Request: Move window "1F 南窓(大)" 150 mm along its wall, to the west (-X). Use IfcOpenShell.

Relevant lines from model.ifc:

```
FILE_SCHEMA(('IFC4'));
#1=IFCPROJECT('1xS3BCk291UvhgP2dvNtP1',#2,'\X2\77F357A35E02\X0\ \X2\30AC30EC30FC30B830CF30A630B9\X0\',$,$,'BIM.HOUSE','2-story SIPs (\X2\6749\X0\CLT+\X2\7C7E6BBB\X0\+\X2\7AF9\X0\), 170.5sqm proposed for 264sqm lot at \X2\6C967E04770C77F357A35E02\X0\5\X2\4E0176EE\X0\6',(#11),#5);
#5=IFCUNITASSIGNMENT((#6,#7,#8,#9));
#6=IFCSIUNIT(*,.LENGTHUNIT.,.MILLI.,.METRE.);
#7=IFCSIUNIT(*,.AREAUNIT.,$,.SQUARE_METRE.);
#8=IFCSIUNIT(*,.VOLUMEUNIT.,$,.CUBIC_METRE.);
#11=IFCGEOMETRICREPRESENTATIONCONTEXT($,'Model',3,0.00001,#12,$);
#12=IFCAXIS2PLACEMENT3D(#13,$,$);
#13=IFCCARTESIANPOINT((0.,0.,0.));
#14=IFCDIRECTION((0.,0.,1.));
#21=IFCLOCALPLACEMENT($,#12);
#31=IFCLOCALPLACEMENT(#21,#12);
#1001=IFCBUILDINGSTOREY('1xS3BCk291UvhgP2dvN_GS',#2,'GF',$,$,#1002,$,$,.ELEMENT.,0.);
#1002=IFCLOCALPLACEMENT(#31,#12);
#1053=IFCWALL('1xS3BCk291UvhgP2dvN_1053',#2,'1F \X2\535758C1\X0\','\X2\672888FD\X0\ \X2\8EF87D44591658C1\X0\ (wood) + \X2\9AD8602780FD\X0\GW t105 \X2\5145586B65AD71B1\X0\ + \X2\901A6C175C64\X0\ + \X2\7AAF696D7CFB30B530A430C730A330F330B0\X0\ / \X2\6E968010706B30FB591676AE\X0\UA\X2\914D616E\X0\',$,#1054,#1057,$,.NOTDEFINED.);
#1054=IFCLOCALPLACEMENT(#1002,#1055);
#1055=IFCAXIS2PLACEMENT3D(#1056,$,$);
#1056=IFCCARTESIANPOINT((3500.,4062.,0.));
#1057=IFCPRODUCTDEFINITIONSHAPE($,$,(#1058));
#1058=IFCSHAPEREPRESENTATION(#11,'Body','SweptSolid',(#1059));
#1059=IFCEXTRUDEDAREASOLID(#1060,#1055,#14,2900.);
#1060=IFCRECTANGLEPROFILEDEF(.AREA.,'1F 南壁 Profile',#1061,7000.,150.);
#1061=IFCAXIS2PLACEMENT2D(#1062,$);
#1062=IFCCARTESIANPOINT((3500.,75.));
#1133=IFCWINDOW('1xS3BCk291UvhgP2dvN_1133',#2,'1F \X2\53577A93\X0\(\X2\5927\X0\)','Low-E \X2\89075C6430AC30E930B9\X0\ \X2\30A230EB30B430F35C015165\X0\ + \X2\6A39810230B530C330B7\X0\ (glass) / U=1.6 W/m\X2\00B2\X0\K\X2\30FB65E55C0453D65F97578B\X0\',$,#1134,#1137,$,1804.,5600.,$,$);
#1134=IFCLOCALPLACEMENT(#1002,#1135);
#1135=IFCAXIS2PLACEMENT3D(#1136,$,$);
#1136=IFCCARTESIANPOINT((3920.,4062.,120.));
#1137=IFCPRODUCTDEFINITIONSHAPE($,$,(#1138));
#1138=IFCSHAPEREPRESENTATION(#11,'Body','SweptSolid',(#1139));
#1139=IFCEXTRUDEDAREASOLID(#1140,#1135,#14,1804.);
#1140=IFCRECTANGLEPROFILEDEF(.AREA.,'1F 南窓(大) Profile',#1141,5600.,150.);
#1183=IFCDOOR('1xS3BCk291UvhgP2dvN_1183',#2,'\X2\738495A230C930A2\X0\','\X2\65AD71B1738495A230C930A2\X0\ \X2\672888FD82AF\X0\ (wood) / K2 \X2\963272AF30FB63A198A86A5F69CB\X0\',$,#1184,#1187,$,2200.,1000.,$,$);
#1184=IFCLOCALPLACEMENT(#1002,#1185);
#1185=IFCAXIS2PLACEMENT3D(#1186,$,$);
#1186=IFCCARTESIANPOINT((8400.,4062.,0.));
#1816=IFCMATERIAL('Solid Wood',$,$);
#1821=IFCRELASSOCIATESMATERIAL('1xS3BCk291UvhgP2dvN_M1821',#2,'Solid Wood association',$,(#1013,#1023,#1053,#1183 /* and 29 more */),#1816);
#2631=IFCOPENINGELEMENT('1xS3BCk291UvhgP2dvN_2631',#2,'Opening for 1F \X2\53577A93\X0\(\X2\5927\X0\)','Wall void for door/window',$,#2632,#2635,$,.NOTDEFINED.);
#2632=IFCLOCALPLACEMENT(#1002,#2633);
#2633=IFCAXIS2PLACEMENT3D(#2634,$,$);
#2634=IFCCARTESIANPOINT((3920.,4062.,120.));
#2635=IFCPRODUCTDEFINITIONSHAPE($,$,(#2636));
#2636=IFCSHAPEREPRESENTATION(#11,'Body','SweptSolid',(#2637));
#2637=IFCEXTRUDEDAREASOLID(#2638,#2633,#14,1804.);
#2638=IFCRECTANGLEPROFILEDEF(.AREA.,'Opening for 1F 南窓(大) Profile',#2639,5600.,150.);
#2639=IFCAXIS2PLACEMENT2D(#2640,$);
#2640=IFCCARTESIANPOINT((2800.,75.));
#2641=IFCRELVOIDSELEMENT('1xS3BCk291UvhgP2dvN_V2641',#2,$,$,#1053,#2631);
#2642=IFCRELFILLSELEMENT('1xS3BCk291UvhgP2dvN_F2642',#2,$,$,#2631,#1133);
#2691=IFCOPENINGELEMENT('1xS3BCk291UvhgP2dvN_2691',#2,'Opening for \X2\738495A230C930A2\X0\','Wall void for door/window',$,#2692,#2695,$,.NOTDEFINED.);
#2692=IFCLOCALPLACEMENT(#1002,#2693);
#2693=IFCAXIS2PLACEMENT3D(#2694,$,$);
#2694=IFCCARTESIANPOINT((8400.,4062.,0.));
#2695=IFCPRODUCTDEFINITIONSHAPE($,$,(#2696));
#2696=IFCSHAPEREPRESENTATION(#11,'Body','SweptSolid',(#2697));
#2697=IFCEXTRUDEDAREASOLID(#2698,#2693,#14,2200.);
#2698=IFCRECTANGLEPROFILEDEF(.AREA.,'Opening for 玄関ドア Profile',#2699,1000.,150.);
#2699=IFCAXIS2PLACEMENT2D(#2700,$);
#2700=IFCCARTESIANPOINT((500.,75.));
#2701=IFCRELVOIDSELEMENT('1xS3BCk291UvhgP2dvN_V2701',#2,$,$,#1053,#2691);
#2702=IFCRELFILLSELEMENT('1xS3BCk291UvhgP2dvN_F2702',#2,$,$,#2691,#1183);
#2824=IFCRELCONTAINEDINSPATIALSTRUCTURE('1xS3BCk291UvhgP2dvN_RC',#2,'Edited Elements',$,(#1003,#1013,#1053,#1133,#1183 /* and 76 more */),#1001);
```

```python
import ifcopenshell
import ifcopenshell.api.geometry
import ifcopenshell.util.placement

model = ifcopenshell.open("model.ifc")

window = model.by_id(1133)
opening = window.FillsVoids[0].RelatingOpeningElement
wall = opening.VoidsElements[0].RelatingBuildingElement

wall_matrix = ifcopenshell.util.placement.get_local_placement(wall.ObjectPlacement)
shift = wall_matrix[:3, 0] * -150.0
before = ifcopenshell.util.placement.get_local_placement(window.ObjectPlacement)[:3, 3].copy()

# The window is not placed relative to its opening, so move both.
for product in (opening, window):
    matrix = ifcopenshell.util.placement.get_local_placement(product.ObjectPlacement)
    matrix[:3, 3] += shift
    ifcopenshell.api.geometry.edit_object_placement(model, product=product, matrix=matrix, is_si=False)

after = ifcopenshell.util.placement.get_local_placement(window.ObjectPlacement)[:3, 3]
print("window moved by", (after - before).round(3) + 0.0)

model.write("model_rev.ifc")
```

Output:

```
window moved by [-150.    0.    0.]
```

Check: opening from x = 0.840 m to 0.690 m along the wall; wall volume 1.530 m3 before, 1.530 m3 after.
